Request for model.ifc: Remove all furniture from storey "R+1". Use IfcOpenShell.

First a look at what the model holds.

```python
import ifcopenshell
import ifcopenshell.util.element

model = ifcopenshell.open("model.ifc")
print(model.schema)
storey = next(s for s in model.by_type("IfcBuildingStorey") if s.Name == "R+1")
furniture = [e for e in ifcopenshell.util.element.get_decomposition(storey) if e.is_a("IfcFurnishingElement")]
seen = {}
for e in furniture:
    element_type = ifcopenshell.util.element.get_type(e)
    name = element_type.Name if element_type not in (None, e) else None
    seen[name] = seen.get(name, 0) + 1
for name, count in sorted(seen.items(), key=str):
    print(count, "x", name)
```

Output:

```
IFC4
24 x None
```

```python
import ifcopenshell
import ifcopenshell.api.root
import ifcopenshell.util.element

model = ifcopenshell.open("model.ifc")

storey = next(s for s in model.by_type("IfcBuildingStorey") if s.Name == "R+1")
furniture = [e for e in ifcopenshell.util.element.get_decomposition(storey) if e.is_a("IfcFurnishingElement")]

for e in furniture:
    ifcopenshell.api.root.remove_product(model, product=e)
print(len(furniture), "removed")

model.write("model-out.ifc")
```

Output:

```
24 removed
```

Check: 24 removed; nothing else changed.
